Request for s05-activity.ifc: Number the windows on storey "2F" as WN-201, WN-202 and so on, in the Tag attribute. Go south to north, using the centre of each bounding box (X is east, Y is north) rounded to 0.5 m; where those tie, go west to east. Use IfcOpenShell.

First a look at what the model holds.

```python
import ifcopenshell
import ifcopenshell.util.element
import ifcopenshell.util.placement

model = ifcopenshell.open("s05-activity.ifc")
print(model.schema)
storey = next(s for s in model.by_type("IfcBuildingStorey") if s.Name == "2F")
windows = [e for e in ifcopenshell.util.element.get_decomposition(storey) if e.is_a("IfcWindow")]
for e in sorted(windows, key=lambda e: e.id()):
    origin = ifcopenshell.util.placement.get_local_placement(e.ObjectPlacement)[:3, 3]
    print(e.id(), e.Tag, e.Name, origin.round(2) + 0.0, sep=" | ")
```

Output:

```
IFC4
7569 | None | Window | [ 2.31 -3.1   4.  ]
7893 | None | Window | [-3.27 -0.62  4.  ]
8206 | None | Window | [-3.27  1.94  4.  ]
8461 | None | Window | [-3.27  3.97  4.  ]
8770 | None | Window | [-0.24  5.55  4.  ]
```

```python
import ifcopenshell
import ifcopenshell.geom
import ifcopenshell.util.element
import ifcopenshell.util.shape

model = ifcopenshell.open("s05-activity.ifc")
settings = ifcopenshell.geom.settings()
settings.set("use-world-coords", True)


def centre(element):
    shape = ifcopenshell.geom.create_shape(settings, element)
    return ifcopenshell.util.shape.get_bbox_centroid(shape.geometry)


storey = next(s for s in model.by_type("IfcBuildingStorey") if s.Name == "2F")
windows = [e for e in ifcopenshell.util.element.get_decomposition(storey) if e.is_a("IfcWindow")]

# Insertion points can sit at a corner or the storey origin, so sort by the geometry (in metres).
centres = {e: centre(e) for e in windows}
windows.sort(key=lambda e: (round(centres[e][1] / 0.5), centres[e][0]))

for i, e in enumerate(windows, start=1):
    number = f"WN-2{i:02d}"
    e.Tag = number
    print(e.id(), number)

model.write("s05-activity_edited.ifc")
```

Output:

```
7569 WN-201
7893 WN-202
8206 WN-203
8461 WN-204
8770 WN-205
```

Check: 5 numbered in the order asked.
